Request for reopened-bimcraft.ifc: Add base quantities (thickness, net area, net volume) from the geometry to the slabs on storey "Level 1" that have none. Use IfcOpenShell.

First a look at what the model holds.

```python
import ifcopenshell
import ifcopenshell.util.element
import ifcopenshell.util.unit

model = ifcopenshell.open("reopened-bimcraft.ifc")
print(model.schema)
for unit_type in ("LENGTHUNIT", "AREAUNIT", "VOLUMEUNIT"):
    print(unit_type, ifcopenshell.util.unit.calculate_unit_scale(model, unit_type))
storey = next(s for s in model.by_type("IfcBuildingStorey") if s.Name == "Level 1")
slabs = [e for e in ifcopenshell.util.element.get_decomposition(storey) if e.is_a("IfcSlab")]
for e in sorted(slabs, key=lambda e: e.id()):
    print(e.id(), e.is_a(), e.Name, list(ifcopenshell.util.element.get_psets(e, qtos_only=True)), sep=" | ")
```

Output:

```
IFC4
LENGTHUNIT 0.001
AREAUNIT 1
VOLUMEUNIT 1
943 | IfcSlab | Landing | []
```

```python
import ifcopenshell
import ifcopenshell.api.pset
import ifcopenshell.geom
import ifcopenshell.util.element
import ifcopenshell.util.shape
import ifcopenshell.util.unit

model = ifcopenshell.open("reopened-bimcraft.ifc")
unit_scale = ifcopenshell.util.unit.calculate_unit_scale(model)
area_scale = ifcopenshell.util.unit.calculate_unit_scale(model, "AREAUNIT")
volume_scale = ifcopenshell.util.unit.calculate_unit_scale(model, "VOLUMEUNIT")
settings = ifcopenshell.geom.settings()

storey = next(s for s in model.by_type("IfcBuildingStorey") if s.Name == "Level 1")
slabs = [e for e in ifcopenshell.util.element.get_decomposition(storey) if e.is_a("IfcSlab")]

for e in sorted(slabs, key=lambda e: e.id()):
    if ifcopenshell.util.element.get_psets(e, qtos_only=True, should_inherit=False):
        continue
    # Geometry comes back in metres, in the element's own axes.
    shape = ifcopenshell.geom.create_shape(settings, e)
    values = {
        "Width": ifcopenshell.util.shape.get_z(shape.geometry) / unit_scale,
        "NetArea": ifcopenshell.util.shape.get_footprint_area(shape.geometry) / area_scale,
        "NetVolume": ifcopenshell.util.shape.get_volume(shape.geometry) / volume_scale,
    }
    qto = ifcopenshell.api.pset.add_qto(model, product=e, name="Qto_SlabBaseQuantities")
    ifcopenshell.api.pset.edit_qto(model, qto=qto, properties=values)
    print(e.id(), {k: round(v, 3) for k, v in values.items()})

model.write("reopened-bimcraft-out.ifc")
```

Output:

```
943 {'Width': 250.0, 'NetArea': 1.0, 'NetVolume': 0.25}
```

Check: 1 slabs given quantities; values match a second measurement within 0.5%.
